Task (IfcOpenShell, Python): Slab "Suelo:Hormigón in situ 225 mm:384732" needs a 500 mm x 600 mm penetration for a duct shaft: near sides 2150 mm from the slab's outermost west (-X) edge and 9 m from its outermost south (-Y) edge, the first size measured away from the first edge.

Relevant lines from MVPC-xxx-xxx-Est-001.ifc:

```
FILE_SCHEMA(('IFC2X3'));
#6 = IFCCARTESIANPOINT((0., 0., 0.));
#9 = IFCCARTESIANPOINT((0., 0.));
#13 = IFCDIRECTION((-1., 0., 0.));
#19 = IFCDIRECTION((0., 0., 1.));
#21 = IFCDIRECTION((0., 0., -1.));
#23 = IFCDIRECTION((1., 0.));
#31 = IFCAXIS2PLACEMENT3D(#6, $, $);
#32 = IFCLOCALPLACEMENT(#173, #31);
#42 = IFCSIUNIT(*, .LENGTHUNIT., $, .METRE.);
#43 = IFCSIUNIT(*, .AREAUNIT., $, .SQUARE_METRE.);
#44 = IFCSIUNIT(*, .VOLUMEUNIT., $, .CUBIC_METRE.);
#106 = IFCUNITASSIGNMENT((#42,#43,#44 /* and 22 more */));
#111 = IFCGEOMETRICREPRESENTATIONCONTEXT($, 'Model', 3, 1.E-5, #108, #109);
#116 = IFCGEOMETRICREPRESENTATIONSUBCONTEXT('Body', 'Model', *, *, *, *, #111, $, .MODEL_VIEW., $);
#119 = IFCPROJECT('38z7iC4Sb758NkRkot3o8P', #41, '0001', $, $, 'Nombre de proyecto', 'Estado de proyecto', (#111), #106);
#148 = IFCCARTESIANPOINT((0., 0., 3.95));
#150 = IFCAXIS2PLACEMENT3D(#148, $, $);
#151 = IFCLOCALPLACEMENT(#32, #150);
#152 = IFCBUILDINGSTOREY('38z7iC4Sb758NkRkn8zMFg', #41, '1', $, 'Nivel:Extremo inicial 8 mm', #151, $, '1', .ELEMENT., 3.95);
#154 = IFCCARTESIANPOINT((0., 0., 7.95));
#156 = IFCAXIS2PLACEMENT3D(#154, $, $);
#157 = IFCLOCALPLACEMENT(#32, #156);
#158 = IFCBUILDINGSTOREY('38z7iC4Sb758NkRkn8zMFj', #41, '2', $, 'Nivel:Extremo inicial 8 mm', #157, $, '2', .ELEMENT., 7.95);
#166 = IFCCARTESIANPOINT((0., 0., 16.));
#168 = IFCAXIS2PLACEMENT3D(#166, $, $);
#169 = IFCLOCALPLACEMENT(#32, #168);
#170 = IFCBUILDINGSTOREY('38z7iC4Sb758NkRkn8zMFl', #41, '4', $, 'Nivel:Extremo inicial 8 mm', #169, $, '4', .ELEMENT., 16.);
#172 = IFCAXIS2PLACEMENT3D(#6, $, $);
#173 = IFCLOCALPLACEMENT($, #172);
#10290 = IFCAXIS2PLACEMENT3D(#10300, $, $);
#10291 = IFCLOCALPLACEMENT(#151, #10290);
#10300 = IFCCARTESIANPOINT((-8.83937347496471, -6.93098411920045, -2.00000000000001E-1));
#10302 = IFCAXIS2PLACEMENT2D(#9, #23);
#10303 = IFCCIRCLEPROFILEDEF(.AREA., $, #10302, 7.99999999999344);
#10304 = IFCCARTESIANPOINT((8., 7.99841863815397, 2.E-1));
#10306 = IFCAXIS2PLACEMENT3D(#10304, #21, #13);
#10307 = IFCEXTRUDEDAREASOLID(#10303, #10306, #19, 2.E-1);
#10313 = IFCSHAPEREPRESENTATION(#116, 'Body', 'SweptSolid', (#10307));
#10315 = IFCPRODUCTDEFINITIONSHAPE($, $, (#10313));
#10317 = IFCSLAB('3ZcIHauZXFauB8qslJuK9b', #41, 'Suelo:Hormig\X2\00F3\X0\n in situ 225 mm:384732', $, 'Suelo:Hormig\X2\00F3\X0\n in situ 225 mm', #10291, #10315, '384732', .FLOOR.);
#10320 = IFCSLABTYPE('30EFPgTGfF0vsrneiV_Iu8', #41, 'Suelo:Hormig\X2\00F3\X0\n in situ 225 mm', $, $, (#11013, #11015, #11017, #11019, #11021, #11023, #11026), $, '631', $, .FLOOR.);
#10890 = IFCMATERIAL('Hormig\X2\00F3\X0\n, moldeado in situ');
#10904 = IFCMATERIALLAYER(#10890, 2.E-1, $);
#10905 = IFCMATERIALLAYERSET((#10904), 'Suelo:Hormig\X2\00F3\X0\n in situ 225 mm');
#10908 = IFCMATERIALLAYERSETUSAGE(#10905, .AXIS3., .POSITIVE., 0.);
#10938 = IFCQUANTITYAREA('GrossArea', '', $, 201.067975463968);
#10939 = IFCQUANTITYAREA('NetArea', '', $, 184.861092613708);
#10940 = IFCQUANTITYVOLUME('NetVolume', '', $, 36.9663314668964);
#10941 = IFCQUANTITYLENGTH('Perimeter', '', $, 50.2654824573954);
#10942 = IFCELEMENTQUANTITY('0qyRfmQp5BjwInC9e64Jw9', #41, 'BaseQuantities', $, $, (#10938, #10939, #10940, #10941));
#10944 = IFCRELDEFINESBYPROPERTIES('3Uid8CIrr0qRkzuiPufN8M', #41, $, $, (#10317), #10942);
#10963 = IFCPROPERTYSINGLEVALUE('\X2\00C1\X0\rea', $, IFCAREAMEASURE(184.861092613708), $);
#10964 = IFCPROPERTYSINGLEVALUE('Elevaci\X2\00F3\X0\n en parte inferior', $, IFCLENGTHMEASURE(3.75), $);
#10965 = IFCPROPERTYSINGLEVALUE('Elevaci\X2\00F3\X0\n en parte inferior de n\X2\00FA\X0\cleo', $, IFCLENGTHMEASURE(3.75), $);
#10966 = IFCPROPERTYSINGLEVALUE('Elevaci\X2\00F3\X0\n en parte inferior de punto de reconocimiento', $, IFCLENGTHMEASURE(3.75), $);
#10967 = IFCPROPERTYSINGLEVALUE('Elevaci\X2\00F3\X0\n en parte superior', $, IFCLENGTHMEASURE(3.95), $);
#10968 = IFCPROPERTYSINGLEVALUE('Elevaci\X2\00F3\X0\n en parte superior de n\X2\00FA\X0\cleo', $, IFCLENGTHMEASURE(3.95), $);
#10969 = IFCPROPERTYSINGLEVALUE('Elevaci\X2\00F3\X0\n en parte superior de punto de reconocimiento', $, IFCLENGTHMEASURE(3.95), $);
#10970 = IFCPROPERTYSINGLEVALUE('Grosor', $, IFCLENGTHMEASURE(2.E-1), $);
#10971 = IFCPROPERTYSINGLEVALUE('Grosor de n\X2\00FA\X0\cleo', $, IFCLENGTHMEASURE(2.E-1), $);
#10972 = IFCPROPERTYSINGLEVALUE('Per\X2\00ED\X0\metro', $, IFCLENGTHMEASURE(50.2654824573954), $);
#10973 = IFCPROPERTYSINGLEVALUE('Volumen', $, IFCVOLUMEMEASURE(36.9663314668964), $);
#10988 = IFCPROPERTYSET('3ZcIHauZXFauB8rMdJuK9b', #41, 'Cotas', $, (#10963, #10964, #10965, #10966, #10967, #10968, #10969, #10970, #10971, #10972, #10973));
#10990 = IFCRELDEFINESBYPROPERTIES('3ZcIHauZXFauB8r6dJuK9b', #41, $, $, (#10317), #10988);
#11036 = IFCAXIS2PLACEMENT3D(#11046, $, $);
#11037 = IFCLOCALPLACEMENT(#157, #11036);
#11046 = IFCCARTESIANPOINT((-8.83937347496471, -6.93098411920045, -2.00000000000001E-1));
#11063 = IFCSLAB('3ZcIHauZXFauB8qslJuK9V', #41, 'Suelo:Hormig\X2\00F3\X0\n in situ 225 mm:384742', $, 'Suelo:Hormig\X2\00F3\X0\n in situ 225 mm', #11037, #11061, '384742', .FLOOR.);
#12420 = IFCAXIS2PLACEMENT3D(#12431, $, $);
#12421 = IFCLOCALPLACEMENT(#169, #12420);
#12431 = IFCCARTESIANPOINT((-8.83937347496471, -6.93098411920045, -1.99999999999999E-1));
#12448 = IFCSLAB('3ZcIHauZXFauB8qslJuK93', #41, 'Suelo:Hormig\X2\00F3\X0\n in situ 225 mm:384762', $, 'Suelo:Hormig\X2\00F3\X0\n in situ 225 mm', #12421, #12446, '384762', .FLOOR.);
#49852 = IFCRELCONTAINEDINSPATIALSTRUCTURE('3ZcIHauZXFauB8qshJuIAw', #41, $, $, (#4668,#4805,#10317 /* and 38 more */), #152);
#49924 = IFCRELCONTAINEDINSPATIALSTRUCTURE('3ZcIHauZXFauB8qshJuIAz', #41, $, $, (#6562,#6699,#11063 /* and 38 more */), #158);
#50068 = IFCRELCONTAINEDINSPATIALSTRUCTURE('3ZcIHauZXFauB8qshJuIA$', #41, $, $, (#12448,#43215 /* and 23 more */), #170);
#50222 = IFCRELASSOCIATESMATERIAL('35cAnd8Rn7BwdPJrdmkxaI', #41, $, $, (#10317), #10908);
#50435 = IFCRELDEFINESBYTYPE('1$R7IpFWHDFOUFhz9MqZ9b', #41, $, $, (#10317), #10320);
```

```python
import numpy as np
import ifcopenshell
import ifcopenshell.api.feature
import ifcopenshell.api.geometry
import ifcopenshell.api.pset
import ifcopenshell.api.root
import ifcopenshell.geom
import ifcopenshell.util.element
import ifcopenshell.util.placement
import ifcopenshell.util.representation
import ifcopenshell.util.shape
import ifcopenshell.util.unit

model = ifcopenshell.open("MVPC-xxx-xxx-Est-001.ifc")
unit_scale = ifcopenshell.util.unit.calculate_unit_scale(model)
area_scale = ifcopenshell.util.unit.calculate_unit_scale(model, "AREAUNIT")
volume_scale = ifcopenshell.util.unit.calculate_unit_scale(model, "VOLUMEUNIT")
settings = ifcopenshell.geom.settings()


def volume(element):
    """Net volume in cubic metres, openings subtracted."""
    shape = ifcopenshell.geom.create_shape(settings, element)
    return ifcopenshell.util.shape.get_volume(shape.geometry)


slab = model.by_id(10317)
before = volume(slab)

# Extent in the slab's own axes, in metres. The edges named are its -X and -Y sides.
slab_shape = ifcopenshell.geom.create_shape(settings, slab)
vertices = ifcopenshell.util.shape.get_vertices(slab_shape.geometry)
x_min, y_min, bottom = vertices.min(axis=0)
top = vertices[:, 2].max()

opening = ifcopenshell.api.root.create_entity(model, ifc_class="IfcOpeningElement", name="Duct shaft opening")
context = ifcopenshell.util.representation.get_context(model, "Model", "Body", "MODEL_VIEW")
width, depth = 0.5, 0.6
outline = [(0.0, 0.0), (width, 0.0), (width, depth), (0.0, depth), (0.0, 0.0)]
# Overshoot both faces by 50 mm so the cut is clean.
shape = ifcopenshell.api.geometry.add_slab_representation(
    model, context=context, depth=top - bottom + 0.1, polyline=outline
)
ifcopenshell.api.geometry.assign_representation(model, product=opening, representation=shape)

matrix = ifcopenshell.util.placement.get_local_placement(slab.ObjectPlacement)
matrix[:, 3] = matrix @ np.append(np.array([x_min + 2.15, y_min + 9, bottom - 0.05]) / unit_scale, 1.0)
ifcopenshell.api.geometry.edit_object_placement(model, product=opening, matrix=matrix, is_si=False)
ifcopenshell.api.feature.add_feature(model, feature=opening, element=slab)

after = volume(slab)

# Update the slab's stored quantities.
qto = model.by_id(ifcopenshell.util.element.get_pset(slab, "BaseQuantities", should_inherit=False)["id"])
ifcopenshell.api.pset.edit_qto(model, qto=qto, properties={
    "NetArea": after / (top - bottom) / area_scale,
    "NetVolume": after / volume_scale,
})
pset = model.by_id(ifcopenshell.util.element.get_pset(slab, "Cotas", should_inherit=False)["id"])
ifcopenshell.api.pset.edit_pset(model, pset=pset, properties={
    "Área": model.create_entity("IfcAreaMeasure", after / (top - bottom) / area_scale),
    "Volumen": model.create_entity("IfcVolumeMeasure", after / volume_scale),
})

print(f"slab volume {before:.3f} -> {after:.3f} m3")

model.write("MVPC-xxx-xxx-Est-001_edited.ifc")
```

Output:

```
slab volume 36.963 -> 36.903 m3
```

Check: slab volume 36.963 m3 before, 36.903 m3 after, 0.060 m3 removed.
